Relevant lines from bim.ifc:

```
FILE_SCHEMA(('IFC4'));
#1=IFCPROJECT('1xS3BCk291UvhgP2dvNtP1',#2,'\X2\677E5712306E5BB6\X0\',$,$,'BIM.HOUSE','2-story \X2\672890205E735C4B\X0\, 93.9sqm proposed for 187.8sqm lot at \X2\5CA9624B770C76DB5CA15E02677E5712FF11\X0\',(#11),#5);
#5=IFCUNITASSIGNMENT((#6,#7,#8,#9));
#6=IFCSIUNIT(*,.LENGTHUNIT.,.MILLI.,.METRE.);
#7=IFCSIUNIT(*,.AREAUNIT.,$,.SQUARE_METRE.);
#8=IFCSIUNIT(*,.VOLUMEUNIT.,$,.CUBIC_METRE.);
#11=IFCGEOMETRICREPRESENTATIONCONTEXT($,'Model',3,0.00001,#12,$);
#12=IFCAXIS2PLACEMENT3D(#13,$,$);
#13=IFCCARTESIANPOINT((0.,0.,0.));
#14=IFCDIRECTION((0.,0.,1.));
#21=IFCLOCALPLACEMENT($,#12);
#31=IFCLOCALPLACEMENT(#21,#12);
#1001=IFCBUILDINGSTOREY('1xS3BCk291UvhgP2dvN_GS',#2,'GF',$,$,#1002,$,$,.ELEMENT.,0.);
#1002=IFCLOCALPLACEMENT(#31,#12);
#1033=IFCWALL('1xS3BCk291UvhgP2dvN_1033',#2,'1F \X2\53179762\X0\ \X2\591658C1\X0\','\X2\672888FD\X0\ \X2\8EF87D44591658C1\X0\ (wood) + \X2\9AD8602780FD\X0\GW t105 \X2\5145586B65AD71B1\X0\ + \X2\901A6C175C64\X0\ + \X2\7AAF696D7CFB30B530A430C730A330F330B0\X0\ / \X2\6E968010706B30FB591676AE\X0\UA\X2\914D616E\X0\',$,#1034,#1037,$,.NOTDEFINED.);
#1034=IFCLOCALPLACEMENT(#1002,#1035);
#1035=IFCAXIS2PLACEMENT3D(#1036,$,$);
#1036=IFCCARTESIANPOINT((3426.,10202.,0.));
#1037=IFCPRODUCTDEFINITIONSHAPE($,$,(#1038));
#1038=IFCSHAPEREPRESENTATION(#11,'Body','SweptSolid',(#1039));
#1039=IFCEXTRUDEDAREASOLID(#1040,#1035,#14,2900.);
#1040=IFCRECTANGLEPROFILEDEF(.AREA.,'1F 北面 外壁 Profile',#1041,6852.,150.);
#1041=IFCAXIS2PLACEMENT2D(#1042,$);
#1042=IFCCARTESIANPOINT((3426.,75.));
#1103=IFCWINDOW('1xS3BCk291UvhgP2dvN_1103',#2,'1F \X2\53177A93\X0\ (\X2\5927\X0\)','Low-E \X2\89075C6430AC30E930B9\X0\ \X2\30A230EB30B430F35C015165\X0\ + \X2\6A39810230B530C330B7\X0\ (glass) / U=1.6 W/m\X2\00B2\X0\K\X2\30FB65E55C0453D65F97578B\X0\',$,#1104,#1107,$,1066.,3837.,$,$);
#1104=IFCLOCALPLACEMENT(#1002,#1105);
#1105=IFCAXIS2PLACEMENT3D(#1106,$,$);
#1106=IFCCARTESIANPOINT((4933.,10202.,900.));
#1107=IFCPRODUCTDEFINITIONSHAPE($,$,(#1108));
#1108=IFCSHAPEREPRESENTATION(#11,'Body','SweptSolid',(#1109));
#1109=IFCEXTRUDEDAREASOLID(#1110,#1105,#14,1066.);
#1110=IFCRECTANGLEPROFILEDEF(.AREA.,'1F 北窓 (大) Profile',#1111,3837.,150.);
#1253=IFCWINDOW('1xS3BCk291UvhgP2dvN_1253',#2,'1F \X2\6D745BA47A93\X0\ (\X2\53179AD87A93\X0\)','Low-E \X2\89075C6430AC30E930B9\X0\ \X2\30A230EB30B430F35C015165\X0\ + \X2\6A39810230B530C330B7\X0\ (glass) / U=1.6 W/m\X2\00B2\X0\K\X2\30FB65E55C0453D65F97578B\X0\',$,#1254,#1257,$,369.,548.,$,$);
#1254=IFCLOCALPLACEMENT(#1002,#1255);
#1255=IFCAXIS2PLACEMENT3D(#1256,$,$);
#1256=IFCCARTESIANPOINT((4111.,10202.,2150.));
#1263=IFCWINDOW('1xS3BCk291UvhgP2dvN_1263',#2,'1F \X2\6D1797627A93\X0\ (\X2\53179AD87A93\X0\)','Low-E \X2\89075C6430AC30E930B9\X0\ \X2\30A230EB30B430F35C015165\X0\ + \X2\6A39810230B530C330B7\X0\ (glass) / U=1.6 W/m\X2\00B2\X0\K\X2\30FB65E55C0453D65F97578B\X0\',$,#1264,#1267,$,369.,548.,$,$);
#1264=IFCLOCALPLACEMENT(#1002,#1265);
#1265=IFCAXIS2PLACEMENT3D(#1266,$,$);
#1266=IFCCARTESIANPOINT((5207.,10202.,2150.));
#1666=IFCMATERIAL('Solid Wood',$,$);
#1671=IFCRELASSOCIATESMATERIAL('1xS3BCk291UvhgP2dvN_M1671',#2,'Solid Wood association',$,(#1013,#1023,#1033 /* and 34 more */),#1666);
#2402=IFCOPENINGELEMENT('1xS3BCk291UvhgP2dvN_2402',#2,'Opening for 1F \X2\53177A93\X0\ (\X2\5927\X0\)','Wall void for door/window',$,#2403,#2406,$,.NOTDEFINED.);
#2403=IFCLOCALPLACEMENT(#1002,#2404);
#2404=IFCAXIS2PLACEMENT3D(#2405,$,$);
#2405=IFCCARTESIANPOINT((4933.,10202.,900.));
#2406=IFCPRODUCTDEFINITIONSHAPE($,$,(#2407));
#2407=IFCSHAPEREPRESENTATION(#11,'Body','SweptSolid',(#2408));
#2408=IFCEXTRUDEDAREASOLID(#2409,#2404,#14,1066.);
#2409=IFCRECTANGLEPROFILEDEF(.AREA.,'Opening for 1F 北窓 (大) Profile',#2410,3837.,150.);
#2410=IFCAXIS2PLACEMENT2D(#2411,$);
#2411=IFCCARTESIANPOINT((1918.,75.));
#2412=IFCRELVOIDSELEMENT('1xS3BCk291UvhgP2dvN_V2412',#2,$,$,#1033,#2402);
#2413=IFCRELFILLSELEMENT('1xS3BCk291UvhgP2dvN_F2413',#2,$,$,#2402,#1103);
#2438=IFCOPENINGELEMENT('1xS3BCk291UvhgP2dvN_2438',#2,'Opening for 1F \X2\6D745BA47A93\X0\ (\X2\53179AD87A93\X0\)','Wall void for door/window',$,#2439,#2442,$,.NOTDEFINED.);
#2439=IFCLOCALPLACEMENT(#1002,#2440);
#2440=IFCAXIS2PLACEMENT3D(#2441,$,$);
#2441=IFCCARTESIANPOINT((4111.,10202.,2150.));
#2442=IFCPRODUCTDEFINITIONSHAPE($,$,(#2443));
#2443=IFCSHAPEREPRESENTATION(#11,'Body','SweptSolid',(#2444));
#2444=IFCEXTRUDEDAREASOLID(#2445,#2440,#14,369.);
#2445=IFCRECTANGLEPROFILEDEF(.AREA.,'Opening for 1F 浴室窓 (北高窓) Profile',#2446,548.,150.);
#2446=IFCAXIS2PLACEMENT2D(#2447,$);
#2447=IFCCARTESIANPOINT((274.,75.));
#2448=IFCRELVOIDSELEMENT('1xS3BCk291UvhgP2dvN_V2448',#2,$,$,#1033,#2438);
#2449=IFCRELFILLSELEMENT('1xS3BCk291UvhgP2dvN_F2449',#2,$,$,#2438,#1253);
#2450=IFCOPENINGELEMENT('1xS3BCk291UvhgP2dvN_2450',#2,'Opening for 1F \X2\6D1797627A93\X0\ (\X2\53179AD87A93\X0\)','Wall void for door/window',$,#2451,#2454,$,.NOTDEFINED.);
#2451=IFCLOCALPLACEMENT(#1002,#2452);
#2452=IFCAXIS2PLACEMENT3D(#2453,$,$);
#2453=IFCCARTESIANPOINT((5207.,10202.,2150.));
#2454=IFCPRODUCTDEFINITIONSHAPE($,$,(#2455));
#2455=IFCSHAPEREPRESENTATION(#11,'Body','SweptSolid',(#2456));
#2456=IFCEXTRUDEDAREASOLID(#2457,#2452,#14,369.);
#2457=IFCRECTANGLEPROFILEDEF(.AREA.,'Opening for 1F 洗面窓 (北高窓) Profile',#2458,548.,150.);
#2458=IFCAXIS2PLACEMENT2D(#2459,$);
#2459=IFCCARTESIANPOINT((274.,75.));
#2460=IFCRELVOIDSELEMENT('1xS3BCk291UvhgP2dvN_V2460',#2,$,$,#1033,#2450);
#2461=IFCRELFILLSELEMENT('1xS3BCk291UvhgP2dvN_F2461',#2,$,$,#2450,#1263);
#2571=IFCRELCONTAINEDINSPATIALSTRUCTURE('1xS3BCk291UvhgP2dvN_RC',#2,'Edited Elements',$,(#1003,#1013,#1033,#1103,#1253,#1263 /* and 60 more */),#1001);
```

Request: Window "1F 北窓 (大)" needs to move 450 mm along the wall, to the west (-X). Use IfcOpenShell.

```python
import ifcopenshell
import ifcopenshell.api.geometry
import ifcopenshell.util.placement
import ifcopenshell.util.unit

model = ifcopenshell.open("bim.ifc")
unit_scale = ifcopenshell.util.unit.calculate_unit_scale(model)

window = model.by_id(1103)
opening = window.FillsVoids[0].RelatingOpeningElement
wall = opening.VoidsElements[0].RelatingBuildingElement

wall_matrix = ifcopenshell.util.placement.get_local_placement(wall.ObjectPlacement)
shift = wall_matrix[:3, 0] * -0.45 / unit_scale
before = ifcopenshell.util.placement.get_local_placement(window.ObjectPlacement)[:3, 3].copy()

# The window is not placed relative to its opening, so move both.
for product in (opening, window):
    matrix = ifcopenshell.util.placement.get_local_placement(product.ObjectPlacement)
    matrix[:3, 3] += shift
    ifcopenshell.api.geometry.edit_object_placement(model, product=product, matrix=matrix, is_si=False)

after = ifcopenshell.util.placement.get_local_placement(window.ObjectPlacement)[:3, 3]
print("window moved by", (after - before).round(3) + 0.0)

model.write("bim_updated.ifc")
```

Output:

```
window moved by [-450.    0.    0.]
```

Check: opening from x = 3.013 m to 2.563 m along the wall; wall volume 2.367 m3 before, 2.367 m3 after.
